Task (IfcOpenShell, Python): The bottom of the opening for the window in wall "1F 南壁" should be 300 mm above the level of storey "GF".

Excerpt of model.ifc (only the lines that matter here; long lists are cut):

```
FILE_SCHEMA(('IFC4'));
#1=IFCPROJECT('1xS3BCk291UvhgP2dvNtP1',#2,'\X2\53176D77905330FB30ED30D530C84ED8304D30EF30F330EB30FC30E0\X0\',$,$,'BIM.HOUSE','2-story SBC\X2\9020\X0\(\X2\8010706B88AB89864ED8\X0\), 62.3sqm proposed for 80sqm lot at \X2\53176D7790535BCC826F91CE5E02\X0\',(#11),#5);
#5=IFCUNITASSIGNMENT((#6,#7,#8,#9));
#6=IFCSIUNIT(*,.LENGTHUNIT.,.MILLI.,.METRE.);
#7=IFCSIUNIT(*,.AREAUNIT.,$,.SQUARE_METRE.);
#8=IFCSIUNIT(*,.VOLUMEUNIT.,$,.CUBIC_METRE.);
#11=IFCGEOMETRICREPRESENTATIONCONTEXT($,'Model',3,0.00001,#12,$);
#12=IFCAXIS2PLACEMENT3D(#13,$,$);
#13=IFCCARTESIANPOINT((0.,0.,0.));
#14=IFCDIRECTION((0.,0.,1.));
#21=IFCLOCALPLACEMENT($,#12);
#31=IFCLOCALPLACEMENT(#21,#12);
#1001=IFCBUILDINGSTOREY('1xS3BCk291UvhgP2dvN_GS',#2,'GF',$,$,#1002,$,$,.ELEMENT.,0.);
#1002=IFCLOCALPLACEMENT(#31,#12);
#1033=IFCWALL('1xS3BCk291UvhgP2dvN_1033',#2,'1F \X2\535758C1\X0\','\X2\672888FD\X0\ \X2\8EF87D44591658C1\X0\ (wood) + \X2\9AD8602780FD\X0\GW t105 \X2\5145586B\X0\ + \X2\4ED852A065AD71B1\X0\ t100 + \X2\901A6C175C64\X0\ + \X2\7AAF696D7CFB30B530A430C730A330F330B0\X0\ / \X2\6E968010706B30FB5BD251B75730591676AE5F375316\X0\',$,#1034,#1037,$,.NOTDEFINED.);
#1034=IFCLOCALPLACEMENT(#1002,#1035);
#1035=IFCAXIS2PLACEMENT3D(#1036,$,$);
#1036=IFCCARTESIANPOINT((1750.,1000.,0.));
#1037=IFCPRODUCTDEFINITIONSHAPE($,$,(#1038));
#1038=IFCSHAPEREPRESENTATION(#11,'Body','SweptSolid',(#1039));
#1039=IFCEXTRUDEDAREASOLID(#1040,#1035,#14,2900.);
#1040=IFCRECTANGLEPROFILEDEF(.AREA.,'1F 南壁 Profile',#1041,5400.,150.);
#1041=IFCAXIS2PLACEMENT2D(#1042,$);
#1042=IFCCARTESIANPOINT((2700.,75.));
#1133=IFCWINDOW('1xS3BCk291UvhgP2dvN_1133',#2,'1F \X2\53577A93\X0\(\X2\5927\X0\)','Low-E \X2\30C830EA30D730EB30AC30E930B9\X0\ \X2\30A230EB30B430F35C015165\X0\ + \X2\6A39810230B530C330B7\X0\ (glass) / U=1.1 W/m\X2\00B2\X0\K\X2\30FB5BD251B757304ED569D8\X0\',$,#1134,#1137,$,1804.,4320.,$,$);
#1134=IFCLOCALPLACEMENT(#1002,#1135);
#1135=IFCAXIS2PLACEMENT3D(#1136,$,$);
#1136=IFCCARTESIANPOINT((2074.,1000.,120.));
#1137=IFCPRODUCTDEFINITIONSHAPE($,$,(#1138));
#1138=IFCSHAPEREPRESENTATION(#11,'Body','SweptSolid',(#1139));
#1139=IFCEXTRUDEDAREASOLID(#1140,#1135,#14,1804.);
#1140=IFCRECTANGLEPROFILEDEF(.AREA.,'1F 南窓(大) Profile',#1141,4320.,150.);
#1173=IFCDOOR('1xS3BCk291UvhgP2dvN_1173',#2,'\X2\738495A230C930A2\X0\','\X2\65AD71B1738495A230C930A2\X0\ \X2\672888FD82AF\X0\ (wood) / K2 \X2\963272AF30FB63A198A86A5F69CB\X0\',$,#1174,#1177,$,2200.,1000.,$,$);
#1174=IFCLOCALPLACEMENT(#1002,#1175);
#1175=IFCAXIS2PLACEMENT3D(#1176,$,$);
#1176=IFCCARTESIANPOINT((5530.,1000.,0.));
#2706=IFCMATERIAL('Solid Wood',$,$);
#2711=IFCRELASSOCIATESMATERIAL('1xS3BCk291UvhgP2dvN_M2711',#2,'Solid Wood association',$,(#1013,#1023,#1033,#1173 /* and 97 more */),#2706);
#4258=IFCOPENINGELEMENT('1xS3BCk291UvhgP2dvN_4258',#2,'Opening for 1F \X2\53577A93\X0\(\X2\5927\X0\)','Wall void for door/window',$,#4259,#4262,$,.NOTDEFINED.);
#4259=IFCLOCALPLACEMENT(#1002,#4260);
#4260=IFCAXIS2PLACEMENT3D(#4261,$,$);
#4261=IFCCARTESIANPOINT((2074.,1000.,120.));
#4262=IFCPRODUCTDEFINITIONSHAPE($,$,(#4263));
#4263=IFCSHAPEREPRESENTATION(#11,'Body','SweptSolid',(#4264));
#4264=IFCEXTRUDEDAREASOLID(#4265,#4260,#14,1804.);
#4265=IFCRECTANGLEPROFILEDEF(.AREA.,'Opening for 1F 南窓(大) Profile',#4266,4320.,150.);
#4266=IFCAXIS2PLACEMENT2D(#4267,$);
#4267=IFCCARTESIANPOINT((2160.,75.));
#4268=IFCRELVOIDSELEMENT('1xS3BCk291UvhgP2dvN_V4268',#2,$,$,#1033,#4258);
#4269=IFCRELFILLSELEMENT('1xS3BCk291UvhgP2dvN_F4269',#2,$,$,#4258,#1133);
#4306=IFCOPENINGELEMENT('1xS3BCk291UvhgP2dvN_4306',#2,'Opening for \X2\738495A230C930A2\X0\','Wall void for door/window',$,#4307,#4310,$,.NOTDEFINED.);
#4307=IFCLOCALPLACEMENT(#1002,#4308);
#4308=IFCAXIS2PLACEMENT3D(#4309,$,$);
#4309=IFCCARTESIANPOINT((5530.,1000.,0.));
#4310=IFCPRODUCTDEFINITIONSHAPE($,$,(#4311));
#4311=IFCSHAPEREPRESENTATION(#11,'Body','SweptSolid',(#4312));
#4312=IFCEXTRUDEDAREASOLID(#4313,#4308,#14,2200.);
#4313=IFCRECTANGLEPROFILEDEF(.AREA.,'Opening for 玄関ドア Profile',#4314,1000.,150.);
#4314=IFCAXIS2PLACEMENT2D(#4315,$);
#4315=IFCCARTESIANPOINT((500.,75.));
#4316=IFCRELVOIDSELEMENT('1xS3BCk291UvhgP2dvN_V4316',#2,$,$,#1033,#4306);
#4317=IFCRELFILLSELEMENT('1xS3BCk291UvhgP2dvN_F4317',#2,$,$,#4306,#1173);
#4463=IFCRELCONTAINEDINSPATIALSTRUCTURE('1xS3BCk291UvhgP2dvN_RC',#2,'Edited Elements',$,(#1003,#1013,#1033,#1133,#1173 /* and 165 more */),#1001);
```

```python
import numpy as np
import ifcopenshell
import ifcopenshell.api.geometry
import ifcopenshell.geom
import ifcopenshell.util.element
import ifcopenshell.util.placement
import ifcopenshell.util.shape
import ifcopenshell.util.unit

model = ifcopenshell.open("model.ifc")
unit_scale = ifcopenshell.util.unit.calculate_unit_scale(model)

window = model.by_guid("1xS3BCk291UvhgP2dvN_1133")
opening = window.FillsVoids[0].RelatingOpeningElement
storey = ifcopenshell.util.element.get_container(window, ifc_class="IfcBuildingStorey")
level = ifcopenshell.util.placement.get_local_placement(storey.ObjectPlacement)[2, 3]

# The opening's origin need not be at the sill, so measure its lowest point.
shape = ifcopenshell.geom.create_shape(ifcopenshell.geom.settings(), opening)
bottom = ifcopenshell.util.shape.get_shape_bottom_elevation(shape, shape.geometry) / unit_scale
dz = level + 0.3 / unit_scale - bottom

shift = np.array([0.0, 0.0, dz])
# The window is not placed relative to its opening, so move both.
for product in (opening, window):
    matrix = ifcopenshell.util.placement.get_local_placement(product.ObjectPlacement)
    matrix[:3, 3] += shift
    ifcopenshell.api.geometry.edit_object_placement(model, product=product, matrix=matrix, is_si=False)

print(f"moved by {dz * unit_scale:+.3f} m")

model.write("model_updated.ifc")
```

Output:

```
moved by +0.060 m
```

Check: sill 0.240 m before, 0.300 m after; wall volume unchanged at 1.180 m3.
